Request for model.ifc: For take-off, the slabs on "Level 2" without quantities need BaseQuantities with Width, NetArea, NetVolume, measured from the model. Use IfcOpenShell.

First a look at what the model holds.

```python
import ifcopenshell
import ifcopenshell.util.element
import ifcopenshell.util.unit

model = ifcopenshell.open("model.ifc")
print(model.schema)
for unit_type in ("LENGTHUNIT", "AREAUNIT", "VOLUMEUNIT"):
    print(unit_type, ifcopenshell.util.unit.calculate_unit_scale(model, unit_type))
storey = next(s for s in model.by_type("IfcBuildingStorey") if s.Name == "Level 2")
slabs = [e for e in ifcopenshell.util.element.get_decomposition(storey) if e.is_a("IfcSlab")]
for e in sorted(slabs, key=lambda e: e.id()):
    print(e.id(), e.is_a(), e.Name, list(ifcopenshell.util.element.get_psets(e, qtos_only=True)), sep=" | ")
```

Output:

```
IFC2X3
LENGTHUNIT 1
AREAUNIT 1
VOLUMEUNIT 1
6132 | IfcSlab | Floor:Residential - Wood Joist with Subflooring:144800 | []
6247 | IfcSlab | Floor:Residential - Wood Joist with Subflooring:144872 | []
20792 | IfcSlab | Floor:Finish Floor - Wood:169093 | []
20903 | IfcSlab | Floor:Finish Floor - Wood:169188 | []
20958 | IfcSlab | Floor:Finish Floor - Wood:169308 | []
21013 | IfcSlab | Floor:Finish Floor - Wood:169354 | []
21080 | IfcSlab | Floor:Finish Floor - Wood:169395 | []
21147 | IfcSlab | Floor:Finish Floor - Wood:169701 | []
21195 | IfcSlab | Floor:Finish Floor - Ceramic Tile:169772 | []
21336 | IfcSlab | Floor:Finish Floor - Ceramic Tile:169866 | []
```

```python
import ifcopenshell
import ifcopenshell.api.pset
import ifcopenshell.geom
import ifcopenshell.util.element
import ifcopenshell.util.shape
import ifcopenshell.util.unit

model = ifcopenshell.open("model.ifc")
unit_scale = ifcopenshell.util.unit.calculate_unit_scale(model)
area_scale = ifcopenshell.util.unit.calculate_unit_scale(model, "AREAUNIT")
volume_scale = ifcopenshell.util.unit.calculate_unit_scale(model, "VOLUMEUNIT")
settings = ifcopenshell.geom.settings()

storey = next(s for s in model.by_type("IfcBuildingStorey") if s.Name == "Level 2")
slabs = [e for e in ifcopenshell.util.element.get_decomposition(storey) if e.is_a("IfcSlab")]

for e in sorted(slabs, key=lambda e: e.id()):
    if ifcopenshell.util.element.get_psets(e, qtos_only=True, should_inherit=False):
        continue
    # Geometry comes back in metres, in the element's own axes.
    shape = ifcopenshell.geom.create_shape(settings, e)
    values = {
        "Width": ifcopenshell.util.shape.get_z(shape.geometry) / unit_scale,
        "NetArea": ifcopenshell.util.shape.get_footprint_area(shape.geometry) / area_scale,
        "NetVolume": ifcopenshell.util.shape.get_volume(shape.geometry) / volume_scale,
    }
    qto = ifcopenshell.api.pset.add_qto(model, product=e, name="BaseQuantities")
    ifcopenshell.api.pset.edit_qto(model, qto=qto, properties=values)
    print(e.id(), {k: round(v, 3) for k, v in values.items()})

model.write("model_updated.ifc")
```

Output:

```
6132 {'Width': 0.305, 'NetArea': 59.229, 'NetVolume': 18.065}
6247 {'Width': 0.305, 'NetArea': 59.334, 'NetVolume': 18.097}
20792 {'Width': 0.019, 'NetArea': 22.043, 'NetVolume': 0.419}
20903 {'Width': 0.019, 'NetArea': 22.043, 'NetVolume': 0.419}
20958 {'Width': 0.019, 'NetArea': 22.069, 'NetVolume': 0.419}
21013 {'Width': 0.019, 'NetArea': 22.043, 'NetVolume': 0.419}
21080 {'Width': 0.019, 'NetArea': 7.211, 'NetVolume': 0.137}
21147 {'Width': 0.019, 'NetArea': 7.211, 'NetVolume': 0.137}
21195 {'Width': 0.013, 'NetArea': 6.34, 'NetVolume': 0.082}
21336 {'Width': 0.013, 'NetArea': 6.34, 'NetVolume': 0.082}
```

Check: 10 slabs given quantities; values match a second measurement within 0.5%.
